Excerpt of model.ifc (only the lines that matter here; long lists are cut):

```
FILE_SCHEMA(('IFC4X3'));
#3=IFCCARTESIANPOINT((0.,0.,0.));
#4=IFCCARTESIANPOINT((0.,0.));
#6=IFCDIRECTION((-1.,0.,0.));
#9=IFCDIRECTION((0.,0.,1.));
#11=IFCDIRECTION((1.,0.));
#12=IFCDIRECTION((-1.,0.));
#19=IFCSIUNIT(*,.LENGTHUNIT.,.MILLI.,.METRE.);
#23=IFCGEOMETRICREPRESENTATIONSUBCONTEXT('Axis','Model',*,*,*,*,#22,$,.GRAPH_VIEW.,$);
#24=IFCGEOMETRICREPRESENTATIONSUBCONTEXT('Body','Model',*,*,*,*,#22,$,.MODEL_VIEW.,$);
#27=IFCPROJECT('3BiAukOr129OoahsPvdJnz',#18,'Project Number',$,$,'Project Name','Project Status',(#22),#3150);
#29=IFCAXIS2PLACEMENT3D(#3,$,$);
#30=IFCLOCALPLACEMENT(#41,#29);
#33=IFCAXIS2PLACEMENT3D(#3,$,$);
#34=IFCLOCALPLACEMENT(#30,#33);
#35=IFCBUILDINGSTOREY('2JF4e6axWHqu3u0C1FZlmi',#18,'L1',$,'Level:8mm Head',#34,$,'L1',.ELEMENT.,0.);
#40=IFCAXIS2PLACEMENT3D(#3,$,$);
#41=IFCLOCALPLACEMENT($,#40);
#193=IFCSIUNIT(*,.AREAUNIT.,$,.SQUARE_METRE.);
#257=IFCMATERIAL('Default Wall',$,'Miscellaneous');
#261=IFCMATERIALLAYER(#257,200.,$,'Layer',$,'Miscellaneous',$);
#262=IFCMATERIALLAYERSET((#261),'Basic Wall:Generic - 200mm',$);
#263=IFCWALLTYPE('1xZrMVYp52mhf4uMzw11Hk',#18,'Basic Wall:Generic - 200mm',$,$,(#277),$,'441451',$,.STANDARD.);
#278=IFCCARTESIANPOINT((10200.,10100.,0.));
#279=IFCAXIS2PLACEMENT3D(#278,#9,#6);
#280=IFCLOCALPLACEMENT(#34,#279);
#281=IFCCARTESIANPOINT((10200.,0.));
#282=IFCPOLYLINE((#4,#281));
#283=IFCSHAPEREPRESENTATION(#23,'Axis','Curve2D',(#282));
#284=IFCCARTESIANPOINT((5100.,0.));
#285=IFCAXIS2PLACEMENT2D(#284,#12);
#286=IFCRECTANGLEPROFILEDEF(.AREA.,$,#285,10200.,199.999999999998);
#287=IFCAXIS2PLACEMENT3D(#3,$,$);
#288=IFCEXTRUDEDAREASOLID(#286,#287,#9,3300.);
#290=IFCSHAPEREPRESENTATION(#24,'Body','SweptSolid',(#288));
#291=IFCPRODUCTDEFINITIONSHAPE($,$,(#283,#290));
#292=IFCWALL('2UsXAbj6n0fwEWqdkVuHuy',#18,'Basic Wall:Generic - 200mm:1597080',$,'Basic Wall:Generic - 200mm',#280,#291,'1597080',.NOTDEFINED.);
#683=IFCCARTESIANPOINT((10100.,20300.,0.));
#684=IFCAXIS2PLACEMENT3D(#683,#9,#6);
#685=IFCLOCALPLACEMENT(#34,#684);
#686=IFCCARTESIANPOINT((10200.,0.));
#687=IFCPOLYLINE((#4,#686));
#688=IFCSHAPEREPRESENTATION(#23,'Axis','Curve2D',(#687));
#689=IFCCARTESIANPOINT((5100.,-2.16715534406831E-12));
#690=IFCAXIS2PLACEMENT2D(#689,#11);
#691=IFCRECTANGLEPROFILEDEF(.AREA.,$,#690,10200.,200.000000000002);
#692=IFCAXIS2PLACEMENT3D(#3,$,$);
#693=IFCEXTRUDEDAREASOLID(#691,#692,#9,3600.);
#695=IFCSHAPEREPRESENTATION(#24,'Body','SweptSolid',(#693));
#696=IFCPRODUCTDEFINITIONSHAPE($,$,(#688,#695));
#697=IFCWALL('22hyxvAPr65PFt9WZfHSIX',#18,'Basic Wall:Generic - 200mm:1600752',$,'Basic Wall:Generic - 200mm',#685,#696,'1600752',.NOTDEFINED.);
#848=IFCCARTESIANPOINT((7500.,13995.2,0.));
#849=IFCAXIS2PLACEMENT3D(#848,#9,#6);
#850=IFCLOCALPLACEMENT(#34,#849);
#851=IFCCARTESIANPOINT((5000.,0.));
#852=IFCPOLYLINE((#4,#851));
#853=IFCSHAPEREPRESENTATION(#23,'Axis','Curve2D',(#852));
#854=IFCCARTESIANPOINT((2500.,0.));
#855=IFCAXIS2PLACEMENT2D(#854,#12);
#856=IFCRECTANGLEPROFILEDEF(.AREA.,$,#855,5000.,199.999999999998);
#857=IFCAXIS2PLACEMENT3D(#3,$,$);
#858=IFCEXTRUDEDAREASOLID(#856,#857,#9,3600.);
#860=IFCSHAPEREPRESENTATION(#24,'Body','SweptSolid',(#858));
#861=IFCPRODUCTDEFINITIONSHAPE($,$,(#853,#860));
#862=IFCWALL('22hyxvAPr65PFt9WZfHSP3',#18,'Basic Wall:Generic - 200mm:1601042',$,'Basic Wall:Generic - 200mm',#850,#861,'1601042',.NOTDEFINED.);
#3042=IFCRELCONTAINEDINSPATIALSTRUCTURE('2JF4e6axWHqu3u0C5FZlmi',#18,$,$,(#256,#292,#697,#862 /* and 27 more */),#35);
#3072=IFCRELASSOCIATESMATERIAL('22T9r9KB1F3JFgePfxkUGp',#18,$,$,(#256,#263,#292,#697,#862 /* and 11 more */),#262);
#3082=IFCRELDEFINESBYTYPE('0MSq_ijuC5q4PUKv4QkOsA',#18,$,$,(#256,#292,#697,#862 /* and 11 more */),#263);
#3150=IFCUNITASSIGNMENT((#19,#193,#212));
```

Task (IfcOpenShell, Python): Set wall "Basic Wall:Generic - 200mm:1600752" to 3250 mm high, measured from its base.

```python
import ifcopenshell
import ifcopenshell.geom
import ifcopenshell.util.representation
import ifcopenshell.util.shape
import ifcopenshell.util.unit

model = ifcopenshell.open("model.ifc")
unit_scale = ifcopenshell.util.unit.calculate_unit_scale(model)
settings = ifcopenshell.geom.settings()


def volume(element):
    """Net volume in cubic metres, openings subtracted."""
    shape = ifcopenshell.geom.create_shape(settings, element)
    return ifcopenshell.util.shape.get_volume(shape.geometry)


wall = model.by_guid("22hyxvAPr65PFt9WZfHSIX")
before = volume(wall)

body = ifcopenshell.util.representation.get_representation(wall, "Model", "Body")
solid = body.Items[0]
old_height = solid.Depth
solid.Depth = 3.25 / unit_scale
after = volume(wall)

print(f"height {old_height:g} -> {solid.Depth:g}, volume {before:.3f} -> {after:.3f} m3")

model.write("model_v2.ifc")
```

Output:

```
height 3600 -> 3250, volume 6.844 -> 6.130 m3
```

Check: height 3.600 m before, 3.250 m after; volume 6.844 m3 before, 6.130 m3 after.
